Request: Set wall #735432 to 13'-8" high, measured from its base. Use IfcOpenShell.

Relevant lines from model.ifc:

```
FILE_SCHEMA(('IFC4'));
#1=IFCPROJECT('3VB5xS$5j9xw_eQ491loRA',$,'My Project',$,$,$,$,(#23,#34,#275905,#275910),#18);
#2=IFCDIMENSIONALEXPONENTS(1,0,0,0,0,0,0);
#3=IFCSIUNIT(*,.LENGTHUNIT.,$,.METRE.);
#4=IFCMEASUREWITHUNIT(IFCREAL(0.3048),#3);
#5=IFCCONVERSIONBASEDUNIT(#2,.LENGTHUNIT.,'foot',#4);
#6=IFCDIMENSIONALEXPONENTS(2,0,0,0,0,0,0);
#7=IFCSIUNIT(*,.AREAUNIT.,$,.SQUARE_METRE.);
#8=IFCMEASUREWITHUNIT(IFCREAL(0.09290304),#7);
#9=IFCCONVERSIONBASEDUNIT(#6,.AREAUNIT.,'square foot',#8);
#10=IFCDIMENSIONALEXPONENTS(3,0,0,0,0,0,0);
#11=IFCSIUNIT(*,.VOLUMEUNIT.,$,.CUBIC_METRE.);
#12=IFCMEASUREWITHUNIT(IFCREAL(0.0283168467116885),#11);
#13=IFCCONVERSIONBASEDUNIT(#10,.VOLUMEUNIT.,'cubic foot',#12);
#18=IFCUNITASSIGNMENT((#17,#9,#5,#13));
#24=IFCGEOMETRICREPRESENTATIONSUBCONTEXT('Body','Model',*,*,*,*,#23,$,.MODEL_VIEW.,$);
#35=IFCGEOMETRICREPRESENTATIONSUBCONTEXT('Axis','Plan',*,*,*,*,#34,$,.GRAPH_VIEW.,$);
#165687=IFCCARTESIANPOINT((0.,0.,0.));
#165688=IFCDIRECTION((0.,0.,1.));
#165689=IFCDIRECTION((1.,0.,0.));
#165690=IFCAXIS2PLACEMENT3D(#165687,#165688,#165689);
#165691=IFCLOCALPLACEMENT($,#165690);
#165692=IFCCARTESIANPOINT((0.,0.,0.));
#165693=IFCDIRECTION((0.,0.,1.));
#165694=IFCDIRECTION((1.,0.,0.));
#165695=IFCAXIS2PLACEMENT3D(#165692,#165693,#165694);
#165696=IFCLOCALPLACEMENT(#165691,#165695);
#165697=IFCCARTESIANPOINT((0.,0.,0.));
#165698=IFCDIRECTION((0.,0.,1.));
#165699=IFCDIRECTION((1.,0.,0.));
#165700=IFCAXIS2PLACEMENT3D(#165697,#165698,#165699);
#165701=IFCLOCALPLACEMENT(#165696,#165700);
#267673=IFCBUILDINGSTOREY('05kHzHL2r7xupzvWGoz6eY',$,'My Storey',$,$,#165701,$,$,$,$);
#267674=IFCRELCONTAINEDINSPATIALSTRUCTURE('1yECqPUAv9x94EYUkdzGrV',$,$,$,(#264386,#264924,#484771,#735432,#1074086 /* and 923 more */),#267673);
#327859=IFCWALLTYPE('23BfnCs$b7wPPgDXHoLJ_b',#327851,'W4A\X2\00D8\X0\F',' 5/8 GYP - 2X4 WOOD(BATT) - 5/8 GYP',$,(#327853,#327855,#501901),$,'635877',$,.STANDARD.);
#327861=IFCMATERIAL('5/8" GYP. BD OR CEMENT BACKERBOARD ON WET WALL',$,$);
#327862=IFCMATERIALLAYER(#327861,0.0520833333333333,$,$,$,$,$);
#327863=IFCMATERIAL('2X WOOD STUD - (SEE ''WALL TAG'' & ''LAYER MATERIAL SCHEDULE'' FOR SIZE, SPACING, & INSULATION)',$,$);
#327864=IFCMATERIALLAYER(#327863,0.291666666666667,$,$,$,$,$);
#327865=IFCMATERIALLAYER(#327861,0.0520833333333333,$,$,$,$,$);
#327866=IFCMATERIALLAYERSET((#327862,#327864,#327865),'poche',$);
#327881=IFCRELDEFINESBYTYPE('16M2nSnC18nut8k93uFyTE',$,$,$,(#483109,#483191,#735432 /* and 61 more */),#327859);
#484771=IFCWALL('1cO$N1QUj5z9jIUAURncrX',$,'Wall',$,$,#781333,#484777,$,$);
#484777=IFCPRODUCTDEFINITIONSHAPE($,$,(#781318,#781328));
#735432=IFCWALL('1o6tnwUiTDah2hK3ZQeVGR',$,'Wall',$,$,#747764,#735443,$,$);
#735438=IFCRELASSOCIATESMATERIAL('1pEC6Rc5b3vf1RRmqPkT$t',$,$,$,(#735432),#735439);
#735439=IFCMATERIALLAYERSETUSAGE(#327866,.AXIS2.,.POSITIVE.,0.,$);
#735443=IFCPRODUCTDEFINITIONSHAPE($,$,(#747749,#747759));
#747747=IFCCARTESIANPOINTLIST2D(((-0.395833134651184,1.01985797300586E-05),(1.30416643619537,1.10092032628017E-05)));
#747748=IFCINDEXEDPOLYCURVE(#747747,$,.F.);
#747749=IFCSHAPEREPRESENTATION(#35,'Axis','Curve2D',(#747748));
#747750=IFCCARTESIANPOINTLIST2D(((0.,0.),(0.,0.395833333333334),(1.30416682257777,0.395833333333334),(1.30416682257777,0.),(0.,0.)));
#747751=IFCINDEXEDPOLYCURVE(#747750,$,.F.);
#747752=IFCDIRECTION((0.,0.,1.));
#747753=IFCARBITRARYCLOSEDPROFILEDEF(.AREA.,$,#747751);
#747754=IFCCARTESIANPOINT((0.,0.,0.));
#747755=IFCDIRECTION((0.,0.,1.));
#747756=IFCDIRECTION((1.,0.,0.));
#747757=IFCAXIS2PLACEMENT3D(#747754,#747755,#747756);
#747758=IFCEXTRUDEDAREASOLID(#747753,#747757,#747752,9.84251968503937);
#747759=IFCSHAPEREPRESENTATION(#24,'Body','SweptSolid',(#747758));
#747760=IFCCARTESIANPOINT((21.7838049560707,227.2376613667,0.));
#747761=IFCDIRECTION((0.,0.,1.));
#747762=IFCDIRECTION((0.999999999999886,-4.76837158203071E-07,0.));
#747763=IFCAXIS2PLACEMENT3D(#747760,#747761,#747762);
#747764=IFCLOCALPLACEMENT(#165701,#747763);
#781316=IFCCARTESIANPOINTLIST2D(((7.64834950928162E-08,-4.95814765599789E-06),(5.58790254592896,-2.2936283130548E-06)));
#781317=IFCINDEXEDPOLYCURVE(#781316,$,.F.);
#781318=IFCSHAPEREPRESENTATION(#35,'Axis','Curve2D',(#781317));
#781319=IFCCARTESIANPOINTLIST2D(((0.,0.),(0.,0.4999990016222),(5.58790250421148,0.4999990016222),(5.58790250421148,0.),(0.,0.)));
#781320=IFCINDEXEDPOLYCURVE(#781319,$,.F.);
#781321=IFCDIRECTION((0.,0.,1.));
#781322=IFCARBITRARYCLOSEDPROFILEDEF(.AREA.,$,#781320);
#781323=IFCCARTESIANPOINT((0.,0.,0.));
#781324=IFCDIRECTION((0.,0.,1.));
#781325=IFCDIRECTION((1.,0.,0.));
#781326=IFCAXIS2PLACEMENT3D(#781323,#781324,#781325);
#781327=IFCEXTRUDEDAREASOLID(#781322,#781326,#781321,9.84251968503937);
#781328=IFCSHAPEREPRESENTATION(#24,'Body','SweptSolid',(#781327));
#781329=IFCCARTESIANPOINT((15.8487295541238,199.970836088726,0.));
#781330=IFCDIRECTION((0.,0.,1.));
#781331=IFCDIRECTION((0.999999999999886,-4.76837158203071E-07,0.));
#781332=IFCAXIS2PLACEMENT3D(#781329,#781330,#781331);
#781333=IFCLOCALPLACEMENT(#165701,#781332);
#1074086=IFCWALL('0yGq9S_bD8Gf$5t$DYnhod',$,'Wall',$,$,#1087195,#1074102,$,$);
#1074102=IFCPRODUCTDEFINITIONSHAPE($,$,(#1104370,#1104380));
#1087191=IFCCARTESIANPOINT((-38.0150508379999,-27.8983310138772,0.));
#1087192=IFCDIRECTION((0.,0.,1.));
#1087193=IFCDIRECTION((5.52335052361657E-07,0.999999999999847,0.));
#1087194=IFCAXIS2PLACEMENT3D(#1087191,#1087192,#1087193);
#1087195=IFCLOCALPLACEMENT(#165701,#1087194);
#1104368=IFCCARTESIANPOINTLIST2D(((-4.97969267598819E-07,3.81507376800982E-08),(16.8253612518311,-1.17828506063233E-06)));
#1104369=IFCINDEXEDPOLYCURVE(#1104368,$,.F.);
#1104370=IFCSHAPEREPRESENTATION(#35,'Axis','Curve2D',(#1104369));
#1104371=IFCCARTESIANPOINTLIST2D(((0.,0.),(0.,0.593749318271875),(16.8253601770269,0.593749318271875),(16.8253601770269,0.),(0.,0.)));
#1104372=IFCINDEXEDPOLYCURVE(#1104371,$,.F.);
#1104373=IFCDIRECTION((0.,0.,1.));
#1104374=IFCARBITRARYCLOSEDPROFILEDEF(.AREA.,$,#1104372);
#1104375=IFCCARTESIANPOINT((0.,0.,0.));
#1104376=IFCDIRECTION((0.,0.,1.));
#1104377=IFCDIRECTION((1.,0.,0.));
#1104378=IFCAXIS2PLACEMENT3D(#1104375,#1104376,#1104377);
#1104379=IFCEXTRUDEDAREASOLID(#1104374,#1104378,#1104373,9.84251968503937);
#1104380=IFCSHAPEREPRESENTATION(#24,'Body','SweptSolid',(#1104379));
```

```python
import ifcopenshell
import ifcopenshell.geom
import ifcopenshell.util.representation
import ifcopenshell.util.shape
import ifcopenshell.util.unit

model = ifcopenshell.open("model.ifc")
unit_scale = ifcopenshell.util.unit.calculate_unit_scale(model)
settings = ifcopenshell.geom.settings()


def volume(element):
    """Net volume in cubic metres, openings subtracted."""
    shape = ifcopenshell.geom.create_shape(settings, element)
    return ifcopenshell.util.shape.get_volume(shape.geometry)


wall = model.by_id(735432)
before = volume(wall)

body = ifcopenshell.util.representation.get_representation(wall, "Model", "Body")
solid = body.Items[0]
old_height = solid.Depth
solid.Depth = 164 * 0.0254 / unit_scale
after = volume(wall)

print(f"height {old_height:g} -> {solid.Depth:g}, volume {before:.3f} -> {after:.3f} m3")

model.write("model_v2.ifc")
```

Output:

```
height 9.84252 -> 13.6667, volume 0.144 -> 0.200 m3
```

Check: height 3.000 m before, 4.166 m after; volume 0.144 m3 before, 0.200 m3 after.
